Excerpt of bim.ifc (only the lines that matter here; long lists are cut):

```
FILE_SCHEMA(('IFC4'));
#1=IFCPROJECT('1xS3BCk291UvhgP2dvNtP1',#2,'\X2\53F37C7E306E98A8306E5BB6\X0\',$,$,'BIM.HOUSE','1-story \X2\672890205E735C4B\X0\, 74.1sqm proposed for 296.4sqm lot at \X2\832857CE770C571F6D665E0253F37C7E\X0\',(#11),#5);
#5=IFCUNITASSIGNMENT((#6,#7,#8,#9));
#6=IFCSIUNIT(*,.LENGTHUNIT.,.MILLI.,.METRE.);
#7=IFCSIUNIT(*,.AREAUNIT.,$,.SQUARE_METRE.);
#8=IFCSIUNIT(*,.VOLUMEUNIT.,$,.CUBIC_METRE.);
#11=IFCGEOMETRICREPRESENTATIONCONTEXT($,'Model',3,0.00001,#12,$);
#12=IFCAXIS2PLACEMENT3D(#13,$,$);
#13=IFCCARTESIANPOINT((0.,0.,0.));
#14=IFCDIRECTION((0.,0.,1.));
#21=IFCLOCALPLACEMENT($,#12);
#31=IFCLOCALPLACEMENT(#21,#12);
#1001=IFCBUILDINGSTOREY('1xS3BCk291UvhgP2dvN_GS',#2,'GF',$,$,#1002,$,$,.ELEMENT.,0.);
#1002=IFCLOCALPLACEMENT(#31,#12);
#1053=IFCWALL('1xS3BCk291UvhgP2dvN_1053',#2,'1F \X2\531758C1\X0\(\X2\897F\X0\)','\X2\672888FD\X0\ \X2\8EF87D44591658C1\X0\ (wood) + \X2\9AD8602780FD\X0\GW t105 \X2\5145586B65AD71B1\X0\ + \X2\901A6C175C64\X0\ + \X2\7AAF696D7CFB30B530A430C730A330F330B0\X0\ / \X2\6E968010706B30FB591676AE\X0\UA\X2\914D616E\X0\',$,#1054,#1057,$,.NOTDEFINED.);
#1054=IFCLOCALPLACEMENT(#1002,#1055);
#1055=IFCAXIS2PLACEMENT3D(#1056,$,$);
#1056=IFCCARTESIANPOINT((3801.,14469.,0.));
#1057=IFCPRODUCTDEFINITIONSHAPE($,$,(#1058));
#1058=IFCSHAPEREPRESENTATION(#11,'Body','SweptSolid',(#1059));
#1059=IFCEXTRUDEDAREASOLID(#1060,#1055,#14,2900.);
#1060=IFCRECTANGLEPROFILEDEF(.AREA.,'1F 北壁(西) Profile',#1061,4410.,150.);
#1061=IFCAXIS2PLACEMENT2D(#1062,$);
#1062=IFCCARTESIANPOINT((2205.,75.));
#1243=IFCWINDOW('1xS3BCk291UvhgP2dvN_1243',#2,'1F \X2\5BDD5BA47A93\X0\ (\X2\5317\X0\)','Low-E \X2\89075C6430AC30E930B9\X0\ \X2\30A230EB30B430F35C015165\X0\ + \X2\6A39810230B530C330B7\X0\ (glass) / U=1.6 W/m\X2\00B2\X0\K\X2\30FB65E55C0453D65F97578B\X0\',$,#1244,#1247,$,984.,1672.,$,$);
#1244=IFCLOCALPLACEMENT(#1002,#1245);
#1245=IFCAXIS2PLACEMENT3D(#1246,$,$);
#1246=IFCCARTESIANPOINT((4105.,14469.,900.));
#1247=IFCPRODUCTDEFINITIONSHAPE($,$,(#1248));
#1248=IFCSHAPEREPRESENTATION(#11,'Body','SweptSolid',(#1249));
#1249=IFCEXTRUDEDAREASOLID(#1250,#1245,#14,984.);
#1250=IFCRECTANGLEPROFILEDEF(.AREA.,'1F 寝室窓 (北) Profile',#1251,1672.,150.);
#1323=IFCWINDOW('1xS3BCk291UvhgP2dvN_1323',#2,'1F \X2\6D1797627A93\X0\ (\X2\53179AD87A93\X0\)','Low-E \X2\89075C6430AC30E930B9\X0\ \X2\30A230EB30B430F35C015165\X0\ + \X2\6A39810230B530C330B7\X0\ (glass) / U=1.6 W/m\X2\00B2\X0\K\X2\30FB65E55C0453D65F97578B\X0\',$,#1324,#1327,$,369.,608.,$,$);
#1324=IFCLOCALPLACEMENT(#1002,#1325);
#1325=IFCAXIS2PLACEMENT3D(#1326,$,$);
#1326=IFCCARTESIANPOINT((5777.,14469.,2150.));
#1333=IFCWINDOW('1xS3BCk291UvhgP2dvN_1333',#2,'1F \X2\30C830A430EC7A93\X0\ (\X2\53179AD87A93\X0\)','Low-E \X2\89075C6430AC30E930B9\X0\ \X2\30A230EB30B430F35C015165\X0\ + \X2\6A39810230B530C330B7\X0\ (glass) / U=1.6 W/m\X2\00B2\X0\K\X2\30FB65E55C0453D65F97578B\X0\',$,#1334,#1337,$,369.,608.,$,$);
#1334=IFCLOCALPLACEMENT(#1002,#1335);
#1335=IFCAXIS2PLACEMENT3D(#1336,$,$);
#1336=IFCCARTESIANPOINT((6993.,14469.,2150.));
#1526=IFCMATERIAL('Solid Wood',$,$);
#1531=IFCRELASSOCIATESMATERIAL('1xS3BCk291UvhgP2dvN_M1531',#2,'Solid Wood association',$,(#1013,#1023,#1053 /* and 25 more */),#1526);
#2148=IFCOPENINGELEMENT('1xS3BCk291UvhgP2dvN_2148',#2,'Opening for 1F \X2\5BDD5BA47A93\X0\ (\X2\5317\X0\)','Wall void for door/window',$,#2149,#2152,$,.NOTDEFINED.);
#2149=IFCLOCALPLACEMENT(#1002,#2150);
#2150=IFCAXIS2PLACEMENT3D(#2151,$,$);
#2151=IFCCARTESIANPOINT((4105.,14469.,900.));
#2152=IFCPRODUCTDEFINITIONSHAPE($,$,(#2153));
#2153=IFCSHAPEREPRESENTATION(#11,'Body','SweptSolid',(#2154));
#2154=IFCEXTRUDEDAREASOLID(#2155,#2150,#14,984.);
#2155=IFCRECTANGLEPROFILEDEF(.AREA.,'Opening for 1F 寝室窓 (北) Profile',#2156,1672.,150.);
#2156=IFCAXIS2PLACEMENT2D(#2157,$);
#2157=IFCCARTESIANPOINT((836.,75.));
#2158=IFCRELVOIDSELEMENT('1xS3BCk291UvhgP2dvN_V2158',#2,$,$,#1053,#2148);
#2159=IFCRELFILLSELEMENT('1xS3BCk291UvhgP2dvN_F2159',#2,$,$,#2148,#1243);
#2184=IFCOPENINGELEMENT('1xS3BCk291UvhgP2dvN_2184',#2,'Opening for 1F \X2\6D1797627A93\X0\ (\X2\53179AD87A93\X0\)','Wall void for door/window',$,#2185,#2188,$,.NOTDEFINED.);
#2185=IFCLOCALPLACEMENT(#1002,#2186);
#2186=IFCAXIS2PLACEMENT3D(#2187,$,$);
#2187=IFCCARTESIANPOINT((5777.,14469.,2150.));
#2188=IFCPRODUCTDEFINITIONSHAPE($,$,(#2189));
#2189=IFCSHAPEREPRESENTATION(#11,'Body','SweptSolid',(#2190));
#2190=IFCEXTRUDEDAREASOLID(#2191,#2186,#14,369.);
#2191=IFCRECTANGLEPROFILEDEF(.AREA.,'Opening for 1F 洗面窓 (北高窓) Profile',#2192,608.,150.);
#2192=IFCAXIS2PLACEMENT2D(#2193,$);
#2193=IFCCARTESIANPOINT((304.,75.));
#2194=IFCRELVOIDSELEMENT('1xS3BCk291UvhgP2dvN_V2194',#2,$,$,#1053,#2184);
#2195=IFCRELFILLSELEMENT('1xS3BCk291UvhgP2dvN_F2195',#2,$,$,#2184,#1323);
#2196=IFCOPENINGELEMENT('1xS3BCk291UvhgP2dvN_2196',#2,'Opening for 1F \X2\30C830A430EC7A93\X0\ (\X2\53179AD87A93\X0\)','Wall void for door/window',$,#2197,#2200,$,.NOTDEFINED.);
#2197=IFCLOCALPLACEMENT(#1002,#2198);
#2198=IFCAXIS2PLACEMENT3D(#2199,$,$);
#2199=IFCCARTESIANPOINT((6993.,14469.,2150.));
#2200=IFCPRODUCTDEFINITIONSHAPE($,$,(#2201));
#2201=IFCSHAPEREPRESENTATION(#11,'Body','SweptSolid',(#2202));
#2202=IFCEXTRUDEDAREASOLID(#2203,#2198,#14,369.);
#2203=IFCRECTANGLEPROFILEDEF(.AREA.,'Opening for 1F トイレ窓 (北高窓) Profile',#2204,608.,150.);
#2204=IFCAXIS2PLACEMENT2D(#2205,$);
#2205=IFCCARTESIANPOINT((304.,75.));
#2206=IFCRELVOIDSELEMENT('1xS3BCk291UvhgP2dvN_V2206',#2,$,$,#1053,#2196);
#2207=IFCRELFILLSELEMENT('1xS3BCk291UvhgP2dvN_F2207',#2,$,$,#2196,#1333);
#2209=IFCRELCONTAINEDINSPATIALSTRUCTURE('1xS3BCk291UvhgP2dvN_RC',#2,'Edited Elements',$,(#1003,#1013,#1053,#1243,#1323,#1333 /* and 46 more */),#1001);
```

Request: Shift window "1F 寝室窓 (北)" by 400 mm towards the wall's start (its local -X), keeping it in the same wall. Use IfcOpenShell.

```python
import ifcopenshell
import ifcopenshell.api.geometry
import ifcopenshell.util.placement
import ifcopenshell.util.unit

model = ifcopenshell.open("bim.ifc")
unit_scale = ifcopenshell.util.unit.calculate_unit_scale(model)

window = model.by_guid("1xS3BCk291UvhgP2dvN_1243")
opening = window.FillsVoids[0].RelatingOpeningElement
wall = opening.VoidsElements[0].RelatingBuildingElement

wall_matrix = ifcopenshell.util.placement.get_local_placement(wall.ObjectPlacement)
shift = wall_matrix[:3, 0] * -0.4 / unit_scale
before = ifcopenshell.util.placement.get_local_placement(window.ObjectPlacement)[:3, 3].copy()

# The window is not placed relative to its opening, so move both.
for product in (opening, window):
    matrix = ifcopenshell.util.placement.get_local_placement(product.ObjectPlacement)
    matrix[:3, 3] += shift
    ifcopenshell.api.geometry.edit_object_placement(model, product=product, matrix=matrix, is_si=False)

after = ifcopenshell.util.placement.get_local_placement(window.ObjectPlacement)[:3, 3]
print("window moved by", (after - before).round(3) + 0.0)

model.write("bim_v2.ifc")
```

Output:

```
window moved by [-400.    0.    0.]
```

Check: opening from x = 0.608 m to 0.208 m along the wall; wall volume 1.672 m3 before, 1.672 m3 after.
